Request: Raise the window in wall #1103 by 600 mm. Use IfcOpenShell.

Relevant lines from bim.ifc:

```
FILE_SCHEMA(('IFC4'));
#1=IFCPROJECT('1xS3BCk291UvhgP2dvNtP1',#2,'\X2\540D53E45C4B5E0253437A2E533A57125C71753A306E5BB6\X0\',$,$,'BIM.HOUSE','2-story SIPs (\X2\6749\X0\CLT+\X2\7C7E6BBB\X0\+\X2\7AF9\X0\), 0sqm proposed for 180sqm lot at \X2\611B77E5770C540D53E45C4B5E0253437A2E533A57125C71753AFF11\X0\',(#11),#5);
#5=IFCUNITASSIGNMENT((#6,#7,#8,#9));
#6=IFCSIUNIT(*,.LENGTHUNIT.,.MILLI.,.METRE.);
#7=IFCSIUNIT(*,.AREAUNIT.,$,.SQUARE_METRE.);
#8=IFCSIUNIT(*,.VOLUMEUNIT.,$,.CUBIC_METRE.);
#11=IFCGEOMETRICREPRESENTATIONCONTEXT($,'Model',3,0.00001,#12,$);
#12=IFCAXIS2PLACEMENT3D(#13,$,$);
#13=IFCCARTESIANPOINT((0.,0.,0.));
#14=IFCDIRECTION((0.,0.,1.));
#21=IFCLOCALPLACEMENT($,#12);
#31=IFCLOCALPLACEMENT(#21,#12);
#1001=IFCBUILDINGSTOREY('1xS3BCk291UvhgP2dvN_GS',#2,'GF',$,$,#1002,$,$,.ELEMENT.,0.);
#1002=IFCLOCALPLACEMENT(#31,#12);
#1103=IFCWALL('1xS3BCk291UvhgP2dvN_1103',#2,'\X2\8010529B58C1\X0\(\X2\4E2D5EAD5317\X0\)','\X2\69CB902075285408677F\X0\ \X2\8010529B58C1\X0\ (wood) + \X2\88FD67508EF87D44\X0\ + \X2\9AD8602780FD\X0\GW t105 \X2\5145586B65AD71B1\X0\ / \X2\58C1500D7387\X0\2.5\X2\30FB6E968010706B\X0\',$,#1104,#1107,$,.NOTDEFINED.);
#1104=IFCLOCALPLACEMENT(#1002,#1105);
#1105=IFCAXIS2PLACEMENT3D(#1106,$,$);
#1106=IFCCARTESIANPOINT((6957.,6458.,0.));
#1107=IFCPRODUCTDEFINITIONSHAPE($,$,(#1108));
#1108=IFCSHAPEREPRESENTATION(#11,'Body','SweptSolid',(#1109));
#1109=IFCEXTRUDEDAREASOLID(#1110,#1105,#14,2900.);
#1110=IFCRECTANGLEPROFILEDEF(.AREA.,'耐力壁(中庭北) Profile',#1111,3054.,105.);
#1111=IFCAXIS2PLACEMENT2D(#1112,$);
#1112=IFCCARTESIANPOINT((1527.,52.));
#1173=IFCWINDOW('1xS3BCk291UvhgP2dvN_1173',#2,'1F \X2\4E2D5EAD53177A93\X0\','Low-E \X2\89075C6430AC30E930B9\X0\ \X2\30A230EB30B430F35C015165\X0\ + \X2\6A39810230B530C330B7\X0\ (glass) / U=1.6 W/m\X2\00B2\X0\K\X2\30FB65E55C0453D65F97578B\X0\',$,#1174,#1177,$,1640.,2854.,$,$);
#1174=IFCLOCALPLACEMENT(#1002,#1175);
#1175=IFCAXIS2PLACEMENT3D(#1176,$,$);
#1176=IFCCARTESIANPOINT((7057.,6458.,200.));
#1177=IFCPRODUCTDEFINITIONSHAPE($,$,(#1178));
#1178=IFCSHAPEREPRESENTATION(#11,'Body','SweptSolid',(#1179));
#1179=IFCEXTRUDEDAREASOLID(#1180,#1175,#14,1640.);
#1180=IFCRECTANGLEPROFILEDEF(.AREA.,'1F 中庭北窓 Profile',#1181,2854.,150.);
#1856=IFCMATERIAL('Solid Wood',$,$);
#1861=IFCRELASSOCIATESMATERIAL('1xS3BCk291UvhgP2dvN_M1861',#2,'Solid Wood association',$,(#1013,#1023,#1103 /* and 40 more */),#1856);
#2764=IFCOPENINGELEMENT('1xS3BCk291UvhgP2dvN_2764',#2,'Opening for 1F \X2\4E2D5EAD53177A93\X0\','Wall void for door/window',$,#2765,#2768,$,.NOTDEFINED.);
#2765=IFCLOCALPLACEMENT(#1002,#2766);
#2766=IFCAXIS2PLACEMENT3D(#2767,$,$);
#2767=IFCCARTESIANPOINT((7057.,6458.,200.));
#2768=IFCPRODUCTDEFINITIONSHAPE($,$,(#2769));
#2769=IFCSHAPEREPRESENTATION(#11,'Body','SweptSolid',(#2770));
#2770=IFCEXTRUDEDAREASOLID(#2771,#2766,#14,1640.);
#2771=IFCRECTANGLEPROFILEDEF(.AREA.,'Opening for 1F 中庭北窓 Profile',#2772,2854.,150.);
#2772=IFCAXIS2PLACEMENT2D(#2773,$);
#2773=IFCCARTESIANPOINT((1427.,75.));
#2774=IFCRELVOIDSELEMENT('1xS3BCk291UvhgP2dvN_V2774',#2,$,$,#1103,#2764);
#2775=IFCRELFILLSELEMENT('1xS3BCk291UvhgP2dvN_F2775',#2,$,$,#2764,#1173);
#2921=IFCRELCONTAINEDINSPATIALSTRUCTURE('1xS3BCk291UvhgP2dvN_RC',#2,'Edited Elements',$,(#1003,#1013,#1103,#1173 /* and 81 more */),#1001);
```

```python
import numpy as np
import ifcopenshell
import ifcopenshell.api.geometry
import ifcopenshell.util.placement
import ifcopenshell.util.unit

model = ifcopenshell.open("bim.ifc")
unit_scale = ifcopenshell.util.unit.calculate_unit_scale(model)

window = model.by_guid("1xS3BCk291UvhgP2dvN_1173")
opening = window.FillsVoids[0].RelatingOpeningElement
dz = 0.6 / unit_scale

shift = np.array([0.0, 0.0, dz])
# The window is not placed relative to its opening, so move both.
for product in (opening, window):
    matrix = ifcopenshell.util.placement.get_local_placement(product.ObjectPlacement)
    matrix[:3, 3] += shift
    ifcopenshell.api.geometry.edit_object_placement(model, product=product, matrix=matrix, is_si=False)

print(f"moved by {dz * unit_scale:+.3f} m")

model.write("bim-out.ifc")
```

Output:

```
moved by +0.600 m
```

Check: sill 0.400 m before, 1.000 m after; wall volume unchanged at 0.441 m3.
